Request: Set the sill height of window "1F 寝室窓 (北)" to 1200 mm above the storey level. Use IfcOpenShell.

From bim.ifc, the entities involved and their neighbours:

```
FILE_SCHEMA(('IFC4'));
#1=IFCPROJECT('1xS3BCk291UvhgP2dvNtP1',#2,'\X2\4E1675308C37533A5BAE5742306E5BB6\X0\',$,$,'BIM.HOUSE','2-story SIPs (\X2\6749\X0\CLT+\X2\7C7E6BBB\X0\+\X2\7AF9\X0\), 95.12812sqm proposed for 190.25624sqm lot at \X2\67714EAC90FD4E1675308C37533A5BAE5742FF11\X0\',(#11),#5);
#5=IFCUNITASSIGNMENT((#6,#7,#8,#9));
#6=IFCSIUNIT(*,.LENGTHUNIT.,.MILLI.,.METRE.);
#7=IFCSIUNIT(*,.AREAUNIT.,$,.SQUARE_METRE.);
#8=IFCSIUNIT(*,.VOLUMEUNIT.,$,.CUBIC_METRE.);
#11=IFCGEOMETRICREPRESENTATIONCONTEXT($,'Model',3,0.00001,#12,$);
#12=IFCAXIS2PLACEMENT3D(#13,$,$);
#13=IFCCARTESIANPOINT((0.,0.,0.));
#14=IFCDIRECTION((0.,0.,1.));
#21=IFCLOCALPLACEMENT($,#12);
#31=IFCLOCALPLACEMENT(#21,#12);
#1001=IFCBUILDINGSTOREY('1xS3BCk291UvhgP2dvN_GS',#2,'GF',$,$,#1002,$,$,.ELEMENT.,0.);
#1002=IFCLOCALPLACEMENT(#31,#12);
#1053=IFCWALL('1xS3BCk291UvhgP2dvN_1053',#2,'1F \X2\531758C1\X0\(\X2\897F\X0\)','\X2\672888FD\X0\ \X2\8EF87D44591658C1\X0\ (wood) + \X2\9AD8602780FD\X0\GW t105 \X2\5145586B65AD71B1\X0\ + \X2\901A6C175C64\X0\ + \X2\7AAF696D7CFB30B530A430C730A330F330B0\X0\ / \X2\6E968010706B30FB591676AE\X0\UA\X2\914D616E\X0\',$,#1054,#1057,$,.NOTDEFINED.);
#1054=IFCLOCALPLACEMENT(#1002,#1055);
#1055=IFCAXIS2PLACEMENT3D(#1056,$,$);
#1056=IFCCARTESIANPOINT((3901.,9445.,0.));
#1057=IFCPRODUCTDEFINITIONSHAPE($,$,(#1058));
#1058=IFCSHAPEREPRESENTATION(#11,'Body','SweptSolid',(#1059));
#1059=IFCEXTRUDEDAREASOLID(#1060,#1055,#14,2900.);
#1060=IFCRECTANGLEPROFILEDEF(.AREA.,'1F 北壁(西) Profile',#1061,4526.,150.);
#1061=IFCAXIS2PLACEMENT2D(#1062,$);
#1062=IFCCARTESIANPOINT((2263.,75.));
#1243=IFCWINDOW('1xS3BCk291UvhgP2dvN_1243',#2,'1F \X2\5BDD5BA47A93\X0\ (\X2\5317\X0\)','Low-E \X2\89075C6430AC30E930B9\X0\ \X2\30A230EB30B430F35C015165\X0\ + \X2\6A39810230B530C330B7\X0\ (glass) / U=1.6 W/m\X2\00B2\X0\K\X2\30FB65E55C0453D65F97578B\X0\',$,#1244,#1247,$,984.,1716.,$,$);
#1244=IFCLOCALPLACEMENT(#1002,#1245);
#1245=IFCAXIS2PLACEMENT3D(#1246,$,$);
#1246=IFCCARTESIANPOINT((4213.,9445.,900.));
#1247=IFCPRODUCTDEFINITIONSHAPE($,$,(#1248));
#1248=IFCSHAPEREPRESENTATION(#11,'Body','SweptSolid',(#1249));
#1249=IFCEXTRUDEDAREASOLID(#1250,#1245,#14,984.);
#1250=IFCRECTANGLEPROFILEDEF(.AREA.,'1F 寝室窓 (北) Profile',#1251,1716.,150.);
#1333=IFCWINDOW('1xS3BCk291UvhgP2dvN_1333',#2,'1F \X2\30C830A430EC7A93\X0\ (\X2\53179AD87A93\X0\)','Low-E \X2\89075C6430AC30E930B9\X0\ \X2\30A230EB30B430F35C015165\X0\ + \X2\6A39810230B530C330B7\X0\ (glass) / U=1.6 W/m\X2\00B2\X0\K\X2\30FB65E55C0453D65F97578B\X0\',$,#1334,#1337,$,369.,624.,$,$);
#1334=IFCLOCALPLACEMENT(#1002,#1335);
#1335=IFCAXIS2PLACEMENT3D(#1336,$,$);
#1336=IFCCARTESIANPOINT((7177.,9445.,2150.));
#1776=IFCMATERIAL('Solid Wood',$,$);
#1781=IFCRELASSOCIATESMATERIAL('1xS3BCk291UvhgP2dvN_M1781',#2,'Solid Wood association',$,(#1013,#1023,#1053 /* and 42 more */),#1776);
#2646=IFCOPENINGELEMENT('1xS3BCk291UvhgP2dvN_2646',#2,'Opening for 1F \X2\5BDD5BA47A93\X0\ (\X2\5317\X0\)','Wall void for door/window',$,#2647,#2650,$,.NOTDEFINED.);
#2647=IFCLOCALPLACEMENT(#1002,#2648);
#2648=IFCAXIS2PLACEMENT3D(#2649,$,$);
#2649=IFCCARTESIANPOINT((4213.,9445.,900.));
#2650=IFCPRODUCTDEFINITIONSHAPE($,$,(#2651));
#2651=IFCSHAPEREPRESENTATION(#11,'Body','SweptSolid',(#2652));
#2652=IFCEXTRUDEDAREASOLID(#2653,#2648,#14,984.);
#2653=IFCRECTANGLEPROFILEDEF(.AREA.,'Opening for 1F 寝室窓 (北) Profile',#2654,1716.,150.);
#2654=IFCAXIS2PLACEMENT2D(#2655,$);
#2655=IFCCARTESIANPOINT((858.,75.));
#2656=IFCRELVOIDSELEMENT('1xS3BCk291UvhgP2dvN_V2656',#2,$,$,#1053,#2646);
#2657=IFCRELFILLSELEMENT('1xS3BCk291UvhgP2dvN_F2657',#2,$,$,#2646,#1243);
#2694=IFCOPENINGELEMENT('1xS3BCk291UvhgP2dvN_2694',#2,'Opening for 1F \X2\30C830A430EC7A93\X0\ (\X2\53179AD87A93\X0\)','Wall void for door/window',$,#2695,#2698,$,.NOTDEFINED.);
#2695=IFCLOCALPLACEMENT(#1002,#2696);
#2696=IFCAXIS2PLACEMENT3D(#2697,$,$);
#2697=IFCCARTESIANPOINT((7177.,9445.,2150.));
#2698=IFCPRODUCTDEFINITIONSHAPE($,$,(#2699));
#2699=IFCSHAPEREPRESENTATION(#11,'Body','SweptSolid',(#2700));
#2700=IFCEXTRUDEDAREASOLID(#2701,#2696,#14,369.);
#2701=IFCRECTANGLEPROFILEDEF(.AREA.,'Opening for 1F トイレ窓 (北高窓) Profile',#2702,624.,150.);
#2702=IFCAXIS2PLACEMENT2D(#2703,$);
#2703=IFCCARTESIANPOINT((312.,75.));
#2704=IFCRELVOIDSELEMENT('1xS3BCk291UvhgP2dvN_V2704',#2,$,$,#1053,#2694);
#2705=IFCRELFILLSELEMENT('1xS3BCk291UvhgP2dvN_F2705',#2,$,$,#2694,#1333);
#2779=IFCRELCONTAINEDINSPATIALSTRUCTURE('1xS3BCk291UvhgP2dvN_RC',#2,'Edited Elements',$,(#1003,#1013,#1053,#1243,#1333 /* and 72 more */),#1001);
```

```python
import numpy as np
import ifcopenshell
import ifcopenshell.api.geometry
import ifcopenshell.geom
import ifcopenshell.util.element
import ifcopenshell.util.placement
import ifcopenshell.util.shape
import ifcopenshell.util.unit

model = ifcopenshell.open("bim.ifc")
unit_scale = ifcopenshell.util.unit.calculate_unit_scale(model)

window = model.by_id(1243)
opening = window.FillsVoids[0].RelatingOpeningElement
storey = ifcopenshell.util.element.get_container(window, ifc_class="IfcBuildingStorey")
level = ifcopenshell.util.placement.get_local_placement(storey.ObjectPlacement)[2, 3]

# The opening's origin need not be at the sill, so measure its lowest point.
shape = ifcopenshell.geom.create_shape(ifcopenshell.geom.settings(), opening)
bottom = ifcopenshell.util.shape.get_shape_bottom_elevation(shape, shape.geometry) / unit_scale
dz = level + 1200.0 - bottom

shift = np.array([0.0, 0.0, dz])
# The window is not placed relative to its opening, so move both.
for product in (opening, window):
    matrix = ifcopenshell.util.placement.get_local_placement(product.ObjectPlacement)
    matrix[:3, 3] += shift
    ifcopenshell.api.geometry.edit_object_placement(model, product=product, matrix=matrix, is_si=False)

print(f"moved by {dz * unit_scale:+.3f} m")

model.write("bim-out.ifc")
```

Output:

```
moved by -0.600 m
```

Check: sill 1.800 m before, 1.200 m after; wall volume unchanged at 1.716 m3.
